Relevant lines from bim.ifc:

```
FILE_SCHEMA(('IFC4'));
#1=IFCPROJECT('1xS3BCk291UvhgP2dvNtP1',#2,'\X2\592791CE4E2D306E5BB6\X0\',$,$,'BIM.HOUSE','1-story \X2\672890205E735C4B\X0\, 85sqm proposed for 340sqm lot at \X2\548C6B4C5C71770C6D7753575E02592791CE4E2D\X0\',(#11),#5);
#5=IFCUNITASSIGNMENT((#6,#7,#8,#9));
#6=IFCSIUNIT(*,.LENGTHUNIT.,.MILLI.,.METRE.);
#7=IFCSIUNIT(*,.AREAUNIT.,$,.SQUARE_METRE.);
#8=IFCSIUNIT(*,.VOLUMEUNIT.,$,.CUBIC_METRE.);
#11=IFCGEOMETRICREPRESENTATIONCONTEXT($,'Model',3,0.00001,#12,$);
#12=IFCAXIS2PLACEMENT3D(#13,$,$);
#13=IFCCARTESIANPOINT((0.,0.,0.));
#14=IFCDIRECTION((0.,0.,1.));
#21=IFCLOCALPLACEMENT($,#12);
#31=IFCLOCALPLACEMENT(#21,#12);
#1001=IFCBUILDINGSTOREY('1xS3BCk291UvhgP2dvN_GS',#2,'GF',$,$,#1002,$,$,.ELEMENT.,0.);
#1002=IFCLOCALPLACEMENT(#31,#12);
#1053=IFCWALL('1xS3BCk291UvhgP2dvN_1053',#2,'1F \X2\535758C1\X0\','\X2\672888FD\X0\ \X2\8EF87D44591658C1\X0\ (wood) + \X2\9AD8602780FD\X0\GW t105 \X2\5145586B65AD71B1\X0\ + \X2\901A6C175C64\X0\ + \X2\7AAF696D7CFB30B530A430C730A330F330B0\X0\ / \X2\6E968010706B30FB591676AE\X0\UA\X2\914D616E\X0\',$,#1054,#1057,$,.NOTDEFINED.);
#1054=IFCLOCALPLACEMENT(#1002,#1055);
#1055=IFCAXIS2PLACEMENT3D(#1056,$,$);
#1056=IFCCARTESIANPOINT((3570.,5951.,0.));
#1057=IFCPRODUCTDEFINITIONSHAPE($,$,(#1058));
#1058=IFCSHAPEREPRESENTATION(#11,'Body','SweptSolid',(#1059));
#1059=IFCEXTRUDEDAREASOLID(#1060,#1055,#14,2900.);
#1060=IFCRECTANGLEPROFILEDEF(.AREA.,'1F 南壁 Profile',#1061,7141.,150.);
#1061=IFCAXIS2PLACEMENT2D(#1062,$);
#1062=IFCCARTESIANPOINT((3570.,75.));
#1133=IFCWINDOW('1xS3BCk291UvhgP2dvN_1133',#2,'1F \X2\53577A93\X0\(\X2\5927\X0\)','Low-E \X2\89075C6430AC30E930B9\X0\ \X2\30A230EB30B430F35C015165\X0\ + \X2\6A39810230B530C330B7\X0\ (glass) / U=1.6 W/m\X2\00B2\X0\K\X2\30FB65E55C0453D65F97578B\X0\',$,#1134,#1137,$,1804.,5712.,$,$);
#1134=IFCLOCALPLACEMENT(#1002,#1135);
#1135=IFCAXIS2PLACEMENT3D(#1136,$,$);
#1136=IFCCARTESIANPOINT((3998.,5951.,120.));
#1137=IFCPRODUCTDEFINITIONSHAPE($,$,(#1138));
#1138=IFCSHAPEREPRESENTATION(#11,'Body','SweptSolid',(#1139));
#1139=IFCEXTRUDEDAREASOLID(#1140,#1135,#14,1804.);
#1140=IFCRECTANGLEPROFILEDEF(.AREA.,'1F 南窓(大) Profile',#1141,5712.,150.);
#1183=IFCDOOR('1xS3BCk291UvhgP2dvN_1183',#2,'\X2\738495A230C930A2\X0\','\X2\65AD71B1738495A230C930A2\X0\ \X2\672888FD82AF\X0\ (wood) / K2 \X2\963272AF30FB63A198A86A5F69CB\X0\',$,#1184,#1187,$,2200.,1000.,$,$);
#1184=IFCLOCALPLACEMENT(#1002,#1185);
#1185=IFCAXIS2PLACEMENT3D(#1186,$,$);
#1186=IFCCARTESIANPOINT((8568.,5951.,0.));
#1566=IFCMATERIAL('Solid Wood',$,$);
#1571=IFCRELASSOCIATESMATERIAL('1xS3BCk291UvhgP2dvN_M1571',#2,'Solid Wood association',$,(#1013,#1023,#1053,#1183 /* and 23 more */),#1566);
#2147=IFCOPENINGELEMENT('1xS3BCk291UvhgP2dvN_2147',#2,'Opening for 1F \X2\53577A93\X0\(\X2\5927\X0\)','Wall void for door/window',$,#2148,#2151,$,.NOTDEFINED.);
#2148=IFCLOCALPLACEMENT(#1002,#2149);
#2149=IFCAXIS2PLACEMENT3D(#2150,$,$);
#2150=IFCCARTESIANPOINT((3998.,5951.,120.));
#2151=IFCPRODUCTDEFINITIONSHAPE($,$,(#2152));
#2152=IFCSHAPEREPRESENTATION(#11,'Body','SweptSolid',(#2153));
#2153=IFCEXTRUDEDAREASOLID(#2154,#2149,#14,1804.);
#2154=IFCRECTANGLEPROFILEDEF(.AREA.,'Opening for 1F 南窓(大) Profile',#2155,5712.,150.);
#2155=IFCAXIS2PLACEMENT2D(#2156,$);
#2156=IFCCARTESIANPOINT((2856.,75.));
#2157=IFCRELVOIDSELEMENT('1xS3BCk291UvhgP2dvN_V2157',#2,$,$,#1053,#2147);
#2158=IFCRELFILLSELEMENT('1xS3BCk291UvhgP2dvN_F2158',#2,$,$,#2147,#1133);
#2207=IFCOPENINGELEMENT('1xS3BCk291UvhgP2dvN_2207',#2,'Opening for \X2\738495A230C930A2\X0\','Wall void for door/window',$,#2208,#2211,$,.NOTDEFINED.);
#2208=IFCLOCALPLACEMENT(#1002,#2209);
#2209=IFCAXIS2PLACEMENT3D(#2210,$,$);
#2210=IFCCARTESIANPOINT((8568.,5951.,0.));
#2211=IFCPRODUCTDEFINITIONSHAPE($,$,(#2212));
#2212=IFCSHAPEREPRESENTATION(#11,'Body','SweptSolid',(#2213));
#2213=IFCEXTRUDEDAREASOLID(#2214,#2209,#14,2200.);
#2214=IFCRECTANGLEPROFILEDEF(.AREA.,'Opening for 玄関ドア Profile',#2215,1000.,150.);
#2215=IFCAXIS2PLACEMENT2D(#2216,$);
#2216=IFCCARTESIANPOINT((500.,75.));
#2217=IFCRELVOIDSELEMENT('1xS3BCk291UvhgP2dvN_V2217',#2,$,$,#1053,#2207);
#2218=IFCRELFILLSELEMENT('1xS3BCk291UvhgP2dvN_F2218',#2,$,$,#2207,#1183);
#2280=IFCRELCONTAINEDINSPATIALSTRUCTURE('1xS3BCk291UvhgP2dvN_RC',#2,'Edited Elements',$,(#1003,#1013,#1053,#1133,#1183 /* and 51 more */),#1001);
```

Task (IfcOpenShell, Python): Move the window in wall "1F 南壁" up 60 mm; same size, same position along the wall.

```python
import numpy as np
import ifcopenshell
import ifcopenshell.api.geometry
import ifcopenshell.util.placement
import ifcopenshell.util.unit

model = ifcopenshell.open("bim.ifc")
unit_scale = ifcopenshell.util.unit.calculate_unit_scale(model)

window = model.by_id(1133)
opening = window.FillsVoids[0].RelatingOpeningElement
dz = 0.06 / unit_scale

shift = np.array([0.0, 0.0, dz])
# The window is not placed relative to its opening, so move both.
for product in (opening, window):
    matrix = ifcopenshell.util.placement.get_local_placement(product.ObjectPlacement)
    matrix[:3, 3] += shift
    ifcopenshell.api.geometry.edit_object_placement(model, product=product, matrix=matrix, is_si=False)

print(f"moved by {dz * unit_scale:+.3f} m")

model.write("bim_edited.ifc")
```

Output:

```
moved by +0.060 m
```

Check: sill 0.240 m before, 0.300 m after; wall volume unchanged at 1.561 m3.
